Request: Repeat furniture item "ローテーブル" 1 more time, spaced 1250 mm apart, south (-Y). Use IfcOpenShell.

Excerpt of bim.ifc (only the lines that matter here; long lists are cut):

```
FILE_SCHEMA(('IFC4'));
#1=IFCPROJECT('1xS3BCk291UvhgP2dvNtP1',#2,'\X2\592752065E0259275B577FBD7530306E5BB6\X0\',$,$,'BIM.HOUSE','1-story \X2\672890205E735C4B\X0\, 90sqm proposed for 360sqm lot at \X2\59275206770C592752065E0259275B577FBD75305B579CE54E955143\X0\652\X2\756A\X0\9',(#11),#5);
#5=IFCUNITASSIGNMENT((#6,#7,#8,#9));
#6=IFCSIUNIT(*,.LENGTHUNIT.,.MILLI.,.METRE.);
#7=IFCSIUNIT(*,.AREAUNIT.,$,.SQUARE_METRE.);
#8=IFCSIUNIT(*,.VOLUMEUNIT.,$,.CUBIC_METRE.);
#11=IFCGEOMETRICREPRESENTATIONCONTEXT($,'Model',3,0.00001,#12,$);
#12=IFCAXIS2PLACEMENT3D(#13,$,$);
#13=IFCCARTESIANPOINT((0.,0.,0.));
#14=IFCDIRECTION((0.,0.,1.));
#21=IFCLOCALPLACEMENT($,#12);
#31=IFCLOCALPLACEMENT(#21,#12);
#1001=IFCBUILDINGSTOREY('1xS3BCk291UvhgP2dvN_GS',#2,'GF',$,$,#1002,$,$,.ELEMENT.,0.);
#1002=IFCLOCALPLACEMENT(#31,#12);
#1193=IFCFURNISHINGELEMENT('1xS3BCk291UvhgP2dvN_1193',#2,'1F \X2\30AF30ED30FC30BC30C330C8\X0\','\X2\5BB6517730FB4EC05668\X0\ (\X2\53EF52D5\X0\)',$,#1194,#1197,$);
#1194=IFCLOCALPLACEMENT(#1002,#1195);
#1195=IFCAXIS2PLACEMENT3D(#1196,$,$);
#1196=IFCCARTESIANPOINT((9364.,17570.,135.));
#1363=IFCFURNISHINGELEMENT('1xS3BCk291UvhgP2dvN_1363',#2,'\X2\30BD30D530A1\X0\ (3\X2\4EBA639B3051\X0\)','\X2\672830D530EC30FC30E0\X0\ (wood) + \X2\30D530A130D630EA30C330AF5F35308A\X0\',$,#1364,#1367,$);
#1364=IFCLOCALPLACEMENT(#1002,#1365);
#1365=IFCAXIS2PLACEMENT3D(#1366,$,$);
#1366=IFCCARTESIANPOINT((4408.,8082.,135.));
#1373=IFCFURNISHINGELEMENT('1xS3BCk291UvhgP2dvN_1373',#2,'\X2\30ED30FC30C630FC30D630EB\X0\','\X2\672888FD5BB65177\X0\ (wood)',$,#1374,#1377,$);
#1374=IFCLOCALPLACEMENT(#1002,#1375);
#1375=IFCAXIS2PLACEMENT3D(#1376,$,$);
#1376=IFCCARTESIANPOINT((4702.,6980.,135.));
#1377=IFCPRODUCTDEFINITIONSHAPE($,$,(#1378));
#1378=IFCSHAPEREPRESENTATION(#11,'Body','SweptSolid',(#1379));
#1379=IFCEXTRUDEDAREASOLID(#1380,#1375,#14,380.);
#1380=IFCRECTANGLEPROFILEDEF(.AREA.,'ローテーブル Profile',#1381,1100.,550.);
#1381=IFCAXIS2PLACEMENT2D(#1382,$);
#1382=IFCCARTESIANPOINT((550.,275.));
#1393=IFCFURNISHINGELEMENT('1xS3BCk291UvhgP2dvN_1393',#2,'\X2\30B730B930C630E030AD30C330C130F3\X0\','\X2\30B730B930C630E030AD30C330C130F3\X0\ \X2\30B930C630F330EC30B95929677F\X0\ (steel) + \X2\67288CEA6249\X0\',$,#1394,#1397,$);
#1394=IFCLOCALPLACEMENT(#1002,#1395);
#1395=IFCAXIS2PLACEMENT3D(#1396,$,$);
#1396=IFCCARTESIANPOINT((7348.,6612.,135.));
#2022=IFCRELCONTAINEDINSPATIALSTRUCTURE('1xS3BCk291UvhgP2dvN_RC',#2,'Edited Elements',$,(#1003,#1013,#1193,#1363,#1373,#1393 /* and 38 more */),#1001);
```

```python
import numpy as np
import ifcopenshell
import ifcopenshell.api.geometry
import ifcopenshell.api.root
import ifcopenshell.util.element
import ifcopenshell.util.placement
import ifcopenshell.util.unit

model = ifcopenshell.open("bim.ifc")
unit_scale = ifcopenshell.util.unit.calculate_unit_scale(model)


def reuse_history(source, copy):
    """copy_class also copies each property set's owner history, people and application; keep the originals."""
    for rel in copy.IsDefinedBy:
        if rel.is_a("IfcRelDefinesByProperties") and (history := rel.RelatingPropertyDefinition.OwnerHistory):
            rel.RelatingPropertyDefinition.OwnerHistory = source.OwnerHistory
            ifcopenshell.util.element.remove_deep2(model, history)


source = model.by_id(1373)
base = ifcopenshell.util.placement.get_local_placement(source.ObjectPlacement)
step = np.array([0.0, -1.0, 0.0]) * 1.25 / unit_scale

for i in range(1, 2):
    copy = ifcopenshell.api.root.copy_class(model, product=source)
    copy.Representation = ifcopenshell.util.element.copy_deep(
        model, source.Representation, exclude=["IfcGeometricRepresentationContext", "IfcRepresentationMap"]
    )
    reuse_history(source, copy)
    matrix = base.copy()
    matrix[:3, 3] += i * step
    print("added at", matrix[:3, 3].round(3) + 0.0)
    ifcopenshell.api.geometry.edit_object_placement(model, product=copy, matrix=matrix, is_si=False)

model.write("bim-out.ifc")
```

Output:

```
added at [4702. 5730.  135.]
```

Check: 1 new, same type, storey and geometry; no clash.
